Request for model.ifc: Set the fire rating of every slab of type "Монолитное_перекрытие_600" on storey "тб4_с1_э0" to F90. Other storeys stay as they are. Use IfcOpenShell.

First a look at what the model holds.

```python
import ifcopenshell
import ifcopenshell.util.element

model = ifcopenshell.open("model.ifc")
print(model.schema)
storey = next(s for s in model.by_type("IfcBuildingStorey") if s.Name == "тб4_с1_э0")
slabs = [e for e in ifcopenshell.util.element.get_decomposition(storey) if e.is_a("IfcSlab")]
seen = {}
for e in slabs:
    element_type = ifcopenshell.util.element.get_type(e)
    key = (element_type.Name if element_type != e and element_type else None, ifcopenshell.util.element.get_pset(e, "Pset_SlabCommon", "FireRating"))
    seen[key] = seen.get(key, 0) + 1
for (name, value), count in sorted(seen.items(), key=str):
    print(count, "x", name, "|", value)
```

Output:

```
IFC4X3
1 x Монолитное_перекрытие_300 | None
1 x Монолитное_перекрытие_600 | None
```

```python
import ifcopenshell
import ifcopenshell.api.pset
import ifcopenshell.util.element

model = ifcopenshell.open("model.ifc")

storey = next(s for s in model.by_type("IfcBuildingStorey") if s.Name == "тб4_с1_э0")
slabs = [e for e in ifcopenshell.util.element.get_decomposition(storey) if e.is_a("IfcSlab")]

count = 0
for e in slabs:
    element_type = ifcopenshell.util.element.get_type(e)
    if element_type in (None, e) or element_type.Name != "Монолитное_перекрытие_600":
        continue
    # add_pset returns the element's existing set when there is one.
    pset = ifcopenshell.api.pset.add_pset(model, product=e, name="Pset_SlabCommon")
    ifcopenshell.api.pset.edit_pset(model, pset=pset, properties={"FireRating": "F90"})
    count += 1

print(count, "slabs updated")

model.write("model_updated.ifc")
```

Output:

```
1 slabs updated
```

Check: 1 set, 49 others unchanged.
